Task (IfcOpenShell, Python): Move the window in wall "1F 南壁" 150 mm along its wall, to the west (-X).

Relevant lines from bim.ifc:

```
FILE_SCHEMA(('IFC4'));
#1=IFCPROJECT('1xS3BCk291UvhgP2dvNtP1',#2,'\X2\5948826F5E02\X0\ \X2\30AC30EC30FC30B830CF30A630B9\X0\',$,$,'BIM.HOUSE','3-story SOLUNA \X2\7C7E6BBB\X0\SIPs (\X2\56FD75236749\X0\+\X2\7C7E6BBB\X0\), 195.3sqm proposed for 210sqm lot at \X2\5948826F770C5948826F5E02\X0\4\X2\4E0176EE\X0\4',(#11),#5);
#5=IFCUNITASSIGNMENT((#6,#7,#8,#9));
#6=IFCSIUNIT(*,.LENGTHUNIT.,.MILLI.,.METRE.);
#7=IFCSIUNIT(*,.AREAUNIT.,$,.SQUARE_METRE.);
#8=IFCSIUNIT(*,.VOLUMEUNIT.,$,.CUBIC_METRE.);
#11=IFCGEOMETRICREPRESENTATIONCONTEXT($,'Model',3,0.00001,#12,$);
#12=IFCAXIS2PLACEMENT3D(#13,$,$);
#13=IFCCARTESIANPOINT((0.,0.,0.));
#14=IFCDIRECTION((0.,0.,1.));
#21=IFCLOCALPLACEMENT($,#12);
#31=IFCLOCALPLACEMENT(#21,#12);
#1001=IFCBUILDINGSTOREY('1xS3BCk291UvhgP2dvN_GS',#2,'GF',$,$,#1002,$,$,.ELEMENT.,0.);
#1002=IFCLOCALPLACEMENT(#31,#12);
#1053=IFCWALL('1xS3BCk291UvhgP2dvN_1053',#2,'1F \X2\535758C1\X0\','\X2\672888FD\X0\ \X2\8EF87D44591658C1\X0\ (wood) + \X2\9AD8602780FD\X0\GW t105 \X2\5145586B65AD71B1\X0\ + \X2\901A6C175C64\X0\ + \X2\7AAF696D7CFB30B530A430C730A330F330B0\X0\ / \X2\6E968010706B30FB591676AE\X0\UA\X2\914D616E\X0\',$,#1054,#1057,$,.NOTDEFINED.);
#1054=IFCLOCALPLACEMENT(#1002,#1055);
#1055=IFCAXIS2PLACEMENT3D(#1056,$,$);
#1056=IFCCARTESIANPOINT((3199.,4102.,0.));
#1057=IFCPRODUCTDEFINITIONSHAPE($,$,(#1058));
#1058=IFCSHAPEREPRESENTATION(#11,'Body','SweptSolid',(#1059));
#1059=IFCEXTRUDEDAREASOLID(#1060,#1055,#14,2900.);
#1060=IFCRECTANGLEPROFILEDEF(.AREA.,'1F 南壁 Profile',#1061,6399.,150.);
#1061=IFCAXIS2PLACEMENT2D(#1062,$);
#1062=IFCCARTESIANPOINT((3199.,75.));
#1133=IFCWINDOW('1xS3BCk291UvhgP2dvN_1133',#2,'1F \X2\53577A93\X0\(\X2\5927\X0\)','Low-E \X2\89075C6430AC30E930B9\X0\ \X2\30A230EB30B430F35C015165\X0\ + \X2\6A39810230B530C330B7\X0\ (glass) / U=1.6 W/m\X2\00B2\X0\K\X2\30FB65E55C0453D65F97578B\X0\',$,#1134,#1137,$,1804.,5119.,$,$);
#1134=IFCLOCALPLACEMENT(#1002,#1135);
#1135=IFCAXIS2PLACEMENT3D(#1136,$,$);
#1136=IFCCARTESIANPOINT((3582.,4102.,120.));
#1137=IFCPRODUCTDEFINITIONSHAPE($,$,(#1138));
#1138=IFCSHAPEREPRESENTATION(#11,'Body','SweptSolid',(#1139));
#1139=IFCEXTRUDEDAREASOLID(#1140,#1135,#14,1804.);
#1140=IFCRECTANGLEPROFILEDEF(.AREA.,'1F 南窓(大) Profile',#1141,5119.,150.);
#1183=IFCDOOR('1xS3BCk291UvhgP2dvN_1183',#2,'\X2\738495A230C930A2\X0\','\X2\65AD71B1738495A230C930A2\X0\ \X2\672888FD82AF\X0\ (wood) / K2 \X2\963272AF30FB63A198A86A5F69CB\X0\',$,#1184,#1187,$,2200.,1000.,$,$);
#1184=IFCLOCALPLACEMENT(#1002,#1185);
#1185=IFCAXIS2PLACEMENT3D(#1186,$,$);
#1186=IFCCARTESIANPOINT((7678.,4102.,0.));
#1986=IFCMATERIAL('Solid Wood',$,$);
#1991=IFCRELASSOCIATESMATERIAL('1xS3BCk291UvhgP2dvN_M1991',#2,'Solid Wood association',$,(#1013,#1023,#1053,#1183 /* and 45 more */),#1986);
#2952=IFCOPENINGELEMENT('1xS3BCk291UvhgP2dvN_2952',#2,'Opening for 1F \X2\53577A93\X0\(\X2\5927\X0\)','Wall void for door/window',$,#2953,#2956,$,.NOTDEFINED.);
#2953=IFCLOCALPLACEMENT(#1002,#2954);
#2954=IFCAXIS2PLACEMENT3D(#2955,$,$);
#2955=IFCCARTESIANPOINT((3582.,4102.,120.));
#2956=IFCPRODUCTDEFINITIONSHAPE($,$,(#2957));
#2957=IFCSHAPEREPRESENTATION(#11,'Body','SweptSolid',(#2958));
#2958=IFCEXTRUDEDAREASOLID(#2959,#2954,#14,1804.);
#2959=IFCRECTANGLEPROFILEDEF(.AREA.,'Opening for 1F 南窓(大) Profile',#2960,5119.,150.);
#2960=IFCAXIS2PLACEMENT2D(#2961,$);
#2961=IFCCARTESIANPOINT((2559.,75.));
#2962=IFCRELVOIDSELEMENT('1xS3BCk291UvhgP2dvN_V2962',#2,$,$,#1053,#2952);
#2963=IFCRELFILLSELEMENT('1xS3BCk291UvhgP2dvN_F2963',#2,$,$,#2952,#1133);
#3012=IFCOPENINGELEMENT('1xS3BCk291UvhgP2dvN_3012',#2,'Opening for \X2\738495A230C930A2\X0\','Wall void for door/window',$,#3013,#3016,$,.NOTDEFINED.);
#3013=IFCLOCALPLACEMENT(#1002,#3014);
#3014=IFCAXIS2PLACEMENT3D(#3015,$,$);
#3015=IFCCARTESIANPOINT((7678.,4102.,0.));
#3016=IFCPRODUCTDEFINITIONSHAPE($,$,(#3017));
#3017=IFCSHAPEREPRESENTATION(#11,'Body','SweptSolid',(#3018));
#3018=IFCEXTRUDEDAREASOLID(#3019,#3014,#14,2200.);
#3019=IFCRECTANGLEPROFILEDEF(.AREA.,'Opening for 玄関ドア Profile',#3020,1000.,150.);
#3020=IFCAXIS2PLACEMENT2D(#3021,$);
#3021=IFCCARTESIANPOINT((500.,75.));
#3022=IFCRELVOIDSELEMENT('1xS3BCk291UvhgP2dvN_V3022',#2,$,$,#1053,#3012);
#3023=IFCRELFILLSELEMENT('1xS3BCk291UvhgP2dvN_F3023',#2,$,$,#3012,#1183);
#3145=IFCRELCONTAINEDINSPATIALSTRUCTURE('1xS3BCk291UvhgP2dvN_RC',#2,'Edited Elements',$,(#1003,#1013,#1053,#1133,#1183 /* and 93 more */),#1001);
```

```python
import ifcopenshell
import ifcopenshell.api.geometry
import ifcopenshell.util.placement
import ifcopenshell.util.unit

model = ifcopenshell.open("bim.ifc")
unit_scale = ifcopenshell.util.unit.calculate_unit_scale(model)

window = model.by_guid("1xS3BCk291UvhgP2dvN_1133")
opening = window.FillsVoids[0].RelatingOpeningElement
wall = opening.VoidsElements[0].RelatingBuildingElement

wall_matrix = ifcopenshell.util.placement.get_local_placement(wall.ObjectPlacement)
shift = wall_matrix[:3, 0] * -0.15 / unit_scale
before = ifcopenshell.util.placement.get_local_placement(window.ObjectPlacement)[:3, 3].copy()

# The window is not placed relative to its opening, so move both.
for product in (opening, window):
    matrix = ifcopenshell.util.placement.get_local_placement(product.ObjectPlacement)
    matrix[:3, 3] += shift
    ifcopenshell.api.geometry.edit_object_placement(model, product=product, matrix=matrix, is_si=False)

after = ifcopenshell.util.placement.get_local_placement(window.ObjectPlacement)[:3, 3]
print("window moved by", (after - before).round(3) + 0.0)

model.write("bim_updated.ifc")
```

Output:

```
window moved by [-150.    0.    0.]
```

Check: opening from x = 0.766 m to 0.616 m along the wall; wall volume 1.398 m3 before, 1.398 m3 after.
